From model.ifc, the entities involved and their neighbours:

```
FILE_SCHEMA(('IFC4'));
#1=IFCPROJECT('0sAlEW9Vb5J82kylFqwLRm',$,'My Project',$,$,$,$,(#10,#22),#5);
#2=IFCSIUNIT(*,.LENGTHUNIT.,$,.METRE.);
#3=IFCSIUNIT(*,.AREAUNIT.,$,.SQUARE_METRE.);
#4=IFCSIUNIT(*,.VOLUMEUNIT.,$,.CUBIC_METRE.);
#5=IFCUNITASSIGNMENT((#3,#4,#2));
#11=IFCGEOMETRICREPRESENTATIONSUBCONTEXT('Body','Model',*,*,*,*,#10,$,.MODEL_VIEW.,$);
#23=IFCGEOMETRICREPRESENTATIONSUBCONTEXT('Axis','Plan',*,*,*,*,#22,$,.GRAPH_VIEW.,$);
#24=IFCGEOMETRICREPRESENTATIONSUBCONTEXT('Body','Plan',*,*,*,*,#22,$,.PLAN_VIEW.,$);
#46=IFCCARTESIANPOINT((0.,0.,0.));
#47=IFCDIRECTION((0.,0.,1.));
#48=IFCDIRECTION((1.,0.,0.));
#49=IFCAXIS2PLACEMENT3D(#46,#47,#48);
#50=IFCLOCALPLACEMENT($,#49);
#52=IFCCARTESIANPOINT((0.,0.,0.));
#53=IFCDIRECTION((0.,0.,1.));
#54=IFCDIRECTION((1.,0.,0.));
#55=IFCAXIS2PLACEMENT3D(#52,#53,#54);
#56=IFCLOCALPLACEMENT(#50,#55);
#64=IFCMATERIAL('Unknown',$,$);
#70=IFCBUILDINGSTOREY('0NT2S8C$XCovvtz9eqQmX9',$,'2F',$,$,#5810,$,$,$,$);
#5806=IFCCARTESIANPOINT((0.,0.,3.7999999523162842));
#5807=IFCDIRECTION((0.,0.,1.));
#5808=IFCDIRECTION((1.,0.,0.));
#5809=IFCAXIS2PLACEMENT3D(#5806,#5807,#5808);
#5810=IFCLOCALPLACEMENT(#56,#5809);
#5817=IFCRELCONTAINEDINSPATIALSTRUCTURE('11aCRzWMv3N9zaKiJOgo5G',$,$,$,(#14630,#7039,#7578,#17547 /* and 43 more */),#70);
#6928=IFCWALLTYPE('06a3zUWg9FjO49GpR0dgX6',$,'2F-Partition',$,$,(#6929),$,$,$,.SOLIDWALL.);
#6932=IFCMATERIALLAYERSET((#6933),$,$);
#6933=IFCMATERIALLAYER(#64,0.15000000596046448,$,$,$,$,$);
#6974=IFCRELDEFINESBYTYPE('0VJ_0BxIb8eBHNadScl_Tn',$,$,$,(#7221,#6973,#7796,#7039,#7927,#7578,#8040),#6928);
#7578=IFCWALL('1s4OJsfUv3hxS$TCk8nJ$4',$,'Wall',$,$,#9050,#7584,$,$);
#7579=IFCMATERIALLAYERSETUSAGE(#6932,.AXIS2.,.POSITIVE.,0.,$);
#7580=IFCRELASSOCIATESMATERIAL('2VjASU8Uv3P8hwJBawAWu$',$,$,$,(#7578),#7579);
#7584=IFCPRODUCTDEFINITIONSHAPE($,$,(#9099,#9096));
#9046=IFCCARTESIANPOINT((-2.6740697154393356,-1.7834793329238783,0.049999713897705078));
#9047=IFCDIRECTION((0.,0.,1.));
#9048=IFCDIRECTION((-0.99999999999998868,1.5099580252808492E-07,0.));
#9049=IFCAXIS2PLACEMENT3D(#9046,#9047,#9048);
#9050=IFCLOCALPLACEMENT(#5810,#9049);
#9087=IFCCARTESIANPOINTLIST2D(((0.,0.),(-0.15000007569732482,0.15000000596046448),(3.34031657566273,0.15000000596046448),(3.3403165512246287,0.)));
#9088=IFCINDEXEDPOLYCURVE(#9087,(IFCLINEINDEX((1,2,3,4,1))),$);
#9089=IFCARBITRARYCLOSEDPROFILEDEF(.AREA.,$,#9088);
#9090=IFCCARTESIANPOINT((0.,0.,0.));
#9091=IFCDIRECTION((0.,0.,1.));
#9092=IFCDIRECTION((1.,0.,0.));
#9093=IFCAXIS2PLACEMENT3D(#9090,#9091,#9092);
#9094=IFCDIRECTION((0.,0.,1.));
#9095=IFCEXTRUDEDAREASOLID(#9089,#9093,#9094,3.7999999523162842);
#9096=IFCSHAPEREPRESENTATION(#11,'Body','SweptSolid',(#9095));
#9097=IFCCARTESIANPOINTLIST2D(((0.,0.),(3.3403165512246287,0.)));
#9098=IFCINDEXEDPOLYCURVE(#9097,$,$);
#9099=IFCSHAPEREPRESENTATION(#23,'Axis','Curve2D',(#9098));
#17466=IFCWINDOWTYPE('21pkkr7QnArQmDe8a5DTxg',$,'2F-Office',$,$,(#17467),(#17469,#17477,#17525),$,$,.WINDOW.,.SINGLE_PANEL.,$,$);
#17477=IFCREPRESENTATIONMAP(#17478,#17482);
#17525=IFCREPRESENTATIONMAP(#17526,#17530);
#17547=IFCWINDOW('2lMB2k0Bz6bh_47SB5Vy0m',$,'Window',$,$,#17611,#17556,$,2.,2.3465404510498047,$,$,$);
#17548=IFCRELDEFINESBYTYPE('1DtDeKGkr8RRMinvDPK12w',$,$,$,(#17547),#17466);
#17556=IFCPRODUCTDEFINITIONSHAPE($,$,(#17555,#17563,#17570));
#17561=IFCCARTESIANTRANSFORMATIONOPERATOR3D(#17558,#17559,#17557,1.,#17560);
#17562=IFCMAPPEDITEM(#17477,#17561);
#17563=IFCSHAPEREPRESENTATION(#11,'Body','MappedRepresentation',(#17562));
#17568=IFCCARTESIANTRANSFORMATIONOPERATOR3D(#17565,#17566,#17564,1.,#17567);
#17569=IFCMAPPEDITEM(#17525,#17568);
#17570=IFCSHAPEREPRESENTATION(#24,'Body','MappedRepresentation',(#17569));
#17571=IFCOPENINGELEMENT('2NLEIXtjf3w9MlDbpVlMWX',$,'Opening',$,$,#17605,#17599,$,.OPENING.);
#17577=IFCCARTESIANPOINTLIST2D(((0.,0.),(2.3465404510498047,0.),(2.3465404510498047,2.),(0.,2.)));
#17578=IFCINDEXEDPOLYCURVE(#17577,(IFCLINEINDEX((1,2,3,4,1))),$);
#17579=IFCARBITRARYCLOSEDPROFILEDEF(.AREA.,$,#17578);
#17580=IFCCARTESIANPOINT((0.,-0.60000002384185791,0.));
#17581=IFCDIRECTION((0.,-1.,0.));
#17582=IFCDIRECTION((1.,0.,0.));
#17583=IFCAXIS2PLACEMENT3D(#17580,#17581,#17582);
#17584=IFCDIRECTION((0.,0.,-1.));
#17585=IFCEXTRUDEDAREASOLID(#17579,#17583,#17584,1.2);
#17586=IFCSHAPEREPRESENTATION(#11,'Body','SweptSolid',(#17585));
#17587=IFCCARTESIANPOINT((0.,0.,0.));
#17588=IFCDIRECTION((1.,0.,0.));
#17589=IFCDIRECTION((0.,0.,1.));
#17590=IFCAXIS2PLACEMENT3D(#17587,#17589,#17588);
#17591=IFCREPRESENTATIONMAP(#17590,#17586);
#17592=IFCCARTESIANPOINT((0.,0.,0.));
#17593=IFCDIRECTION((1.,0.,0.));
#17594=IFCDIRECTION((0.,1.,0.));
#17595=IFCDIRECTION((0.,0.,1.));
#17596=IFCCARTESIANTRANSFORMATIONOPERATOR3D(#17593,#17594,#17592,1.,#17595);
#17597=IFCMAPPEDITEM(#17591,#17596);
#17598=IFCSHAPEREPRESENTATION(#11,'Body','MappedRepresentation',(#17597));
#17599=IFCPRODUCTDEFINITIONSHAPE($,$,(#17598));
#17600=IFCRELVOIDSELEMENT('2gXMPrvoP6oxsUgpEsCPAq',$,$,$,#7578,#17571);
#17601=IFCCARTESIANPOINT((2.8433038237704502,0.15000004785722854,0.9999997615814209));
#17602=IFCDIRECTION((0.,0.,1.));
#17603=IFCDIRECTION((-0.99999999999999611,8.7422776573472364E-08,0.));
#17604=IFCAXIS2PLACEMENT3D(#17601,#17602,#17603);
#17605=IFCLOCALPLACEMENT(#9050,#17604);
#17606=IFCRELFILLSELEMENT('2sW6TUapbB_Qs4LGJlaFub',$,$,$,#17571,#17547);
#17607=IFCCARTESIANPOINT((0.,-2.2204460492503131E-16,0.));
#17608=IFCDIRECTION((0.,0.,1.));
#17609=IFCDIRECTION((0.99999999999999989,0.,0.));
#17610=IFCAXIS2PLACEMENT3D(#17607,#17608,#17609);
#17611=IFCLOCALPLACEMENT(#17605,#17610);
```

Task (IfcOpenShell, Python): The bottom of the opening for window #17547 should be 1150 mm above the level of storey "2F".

```python
import numpy as np
import ifcopenshell
import ifcopenshell.api.geometry
import ifcopenshell.geom
import ifcopenshell.util.element
import ifcopenshell.util.placement
import ifcopenshell.util.shape
import ifcopenshell.util.unit

model = ifcopenshell.open("model.ifc")
unit_scale = ifcopenshell.util.unit.calculate_unit_scale(model)

window = model.by_guid("2lMB2k0Bz6bh_47SB5Vy0m")
opening = window.FillsVoids[0].RelatingOpeningElement
storey = ifcopenshell.util.element.get_container(window, ifc_class="IfcBuildingStorey")
level = ifcopenshell.util.placement.get_local_placement(storey.ObjectPlacement)[2, 3]

# The opening's origin need not be at the sill, so measure its lowest point.
shape = ifcopenshell.geom.create_shape(ifcopenshell.geom.settings(), opening)
bottom = ifcopenshell.util.shape.get_shape_bottom_elevation(shape, shape.geometry) / unit_scale
dz = level + 1.15 - bottom

shift = np.array([0.0, 0.0, dz])
# The window is placed relative to its opening, so it follows when the opening moves.
matrix = ifcopenshell.util.placement.get_local_placement(opening.ObjectPlacement)
matrix[:3, 3] += shift
ifcopenshell.api.geometry.edit_object_placement(
    model, product=opening, matrix=matrix, is_si=False, should_transform_children=True
)

print(f"moved by {dz * unit_scale:+.3f} m")

model.write("model-out.ifc")
```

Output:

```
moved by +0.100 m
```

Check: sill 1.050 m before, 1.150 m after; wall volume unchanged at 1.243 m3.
